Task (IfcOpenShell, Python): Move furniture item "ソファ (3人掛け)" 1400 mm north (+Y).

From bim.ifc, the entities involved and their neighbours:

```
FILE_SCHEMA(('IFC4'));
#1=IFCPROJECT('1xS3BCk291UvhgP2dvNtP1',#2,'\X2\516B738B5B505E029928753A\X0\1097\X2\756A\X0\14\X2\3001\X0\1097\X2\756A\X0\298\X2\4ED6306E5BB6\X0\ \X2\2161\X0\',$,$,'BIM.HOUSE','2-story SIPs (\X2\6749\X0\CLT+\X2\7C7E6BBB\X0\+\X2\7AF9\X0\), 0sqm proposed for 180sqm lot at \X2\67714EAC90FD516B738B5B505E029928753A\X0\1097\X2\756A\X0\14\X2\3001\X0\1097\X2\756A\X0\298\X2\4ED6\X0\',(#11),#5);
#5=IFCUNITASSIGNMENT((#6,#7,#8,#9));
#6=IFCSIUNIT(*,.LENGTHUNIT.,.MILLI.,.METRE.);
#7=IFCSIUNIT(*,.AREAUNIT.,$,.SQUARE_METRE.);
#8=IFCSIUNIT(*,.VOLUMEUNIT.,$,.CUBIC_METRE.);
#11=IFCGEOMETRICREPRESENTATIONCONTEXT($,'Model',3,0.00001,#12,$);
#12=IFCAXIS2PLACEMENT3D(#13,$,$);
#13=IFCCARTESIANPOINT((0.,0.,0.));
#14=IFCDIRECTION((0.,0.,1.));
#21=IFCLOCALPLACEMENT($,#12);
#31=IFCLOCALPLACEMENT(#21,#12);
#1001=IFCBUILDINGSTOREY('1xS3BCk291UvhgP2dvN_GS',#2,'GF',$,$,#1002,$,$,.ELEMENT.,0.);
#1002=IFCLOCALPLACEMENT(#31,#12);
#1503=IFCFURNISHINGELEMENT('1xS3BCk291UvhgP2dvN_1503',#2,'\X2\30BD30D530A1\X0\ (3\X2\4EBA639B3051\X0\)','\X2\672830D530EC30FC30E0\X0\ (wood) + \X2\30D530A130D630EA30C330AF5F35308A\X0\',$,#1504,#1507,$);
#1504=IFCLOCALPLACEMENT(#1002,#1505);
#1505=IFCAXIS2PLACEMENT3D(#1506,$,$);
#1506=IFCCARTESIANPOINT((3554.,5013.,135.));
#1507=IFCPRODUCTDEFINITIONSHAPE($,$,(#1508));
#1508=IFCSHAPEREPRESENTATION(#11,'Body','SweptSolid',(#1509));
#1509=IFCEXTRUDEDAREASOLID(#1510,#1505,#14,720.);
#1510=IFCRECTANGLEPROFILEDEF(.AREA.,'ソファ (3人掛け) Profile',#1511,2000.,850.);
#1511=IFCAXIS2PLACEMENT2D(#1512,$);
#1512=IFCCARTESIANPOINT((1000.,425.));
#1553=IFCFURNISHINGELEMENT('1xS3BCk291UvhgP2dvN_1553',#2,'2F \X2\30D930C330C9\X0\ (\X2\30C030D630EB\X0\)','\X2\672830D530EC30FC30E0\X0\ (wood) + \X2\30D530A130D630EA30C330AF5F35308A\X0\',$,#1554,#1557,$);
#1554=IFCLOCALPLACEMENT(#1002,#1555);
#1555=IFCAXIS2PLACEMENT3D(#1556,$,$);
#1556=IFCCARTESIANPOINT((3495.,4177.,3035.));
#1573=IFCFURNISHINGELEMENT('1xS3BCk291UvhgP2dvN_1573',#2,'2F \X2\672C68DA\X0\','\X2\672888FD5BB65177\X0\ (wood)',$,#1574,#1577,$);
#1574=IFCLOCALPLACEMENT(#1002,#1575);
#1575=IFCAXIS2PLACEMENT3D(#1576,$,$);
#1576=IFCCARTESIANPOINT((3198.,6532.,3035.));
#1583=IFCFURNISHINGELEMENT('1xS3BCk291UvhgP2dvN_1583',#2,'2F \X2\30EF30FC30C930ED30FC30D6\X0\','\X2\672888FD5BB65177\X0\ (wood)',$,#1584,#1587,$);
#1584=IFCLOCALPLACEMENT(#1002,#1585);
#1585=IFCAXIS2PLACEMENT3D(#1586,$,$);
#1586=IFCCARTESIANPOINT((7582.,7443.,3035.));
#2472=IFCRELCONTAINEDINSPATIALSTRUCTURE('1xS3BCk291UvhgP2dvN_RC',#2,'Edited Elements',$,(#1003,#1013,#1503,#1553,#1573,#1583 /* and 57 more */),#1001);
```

```python
import ifcopenshell
import ifcopenshell.api.geometry
import ifcopenshell.util.placement
import ifcopenshell.util.unit

model = ifcopenshell.open("bim.ifc")
unit_scale = ifcopenshell.util.unit.calculate_unit_scale(model)

item = model.by_id(1503)
matrix = ifcopenshell.util.placement.get_local_placement(item.ObjectPlacement)
matrix[1, 3] += 1.4 / unit_scale
ifcopenshell.api.geometry.edit_object_placement(model, product=item, matrix=matrix, is_si=False)

print(ifcopenshell.util.placement.get_local_placement(item.ObjectPlacement).round(3) + 0.0)

model.write("bim_rev.ifc")
```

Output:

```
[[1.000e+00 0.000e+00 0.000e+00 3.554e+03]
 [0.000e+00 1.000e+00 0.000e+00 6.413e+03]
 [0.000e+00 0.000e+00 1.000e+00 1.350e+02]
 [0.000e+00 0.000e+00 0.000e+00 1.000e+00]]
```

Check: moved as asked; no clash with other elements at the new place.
